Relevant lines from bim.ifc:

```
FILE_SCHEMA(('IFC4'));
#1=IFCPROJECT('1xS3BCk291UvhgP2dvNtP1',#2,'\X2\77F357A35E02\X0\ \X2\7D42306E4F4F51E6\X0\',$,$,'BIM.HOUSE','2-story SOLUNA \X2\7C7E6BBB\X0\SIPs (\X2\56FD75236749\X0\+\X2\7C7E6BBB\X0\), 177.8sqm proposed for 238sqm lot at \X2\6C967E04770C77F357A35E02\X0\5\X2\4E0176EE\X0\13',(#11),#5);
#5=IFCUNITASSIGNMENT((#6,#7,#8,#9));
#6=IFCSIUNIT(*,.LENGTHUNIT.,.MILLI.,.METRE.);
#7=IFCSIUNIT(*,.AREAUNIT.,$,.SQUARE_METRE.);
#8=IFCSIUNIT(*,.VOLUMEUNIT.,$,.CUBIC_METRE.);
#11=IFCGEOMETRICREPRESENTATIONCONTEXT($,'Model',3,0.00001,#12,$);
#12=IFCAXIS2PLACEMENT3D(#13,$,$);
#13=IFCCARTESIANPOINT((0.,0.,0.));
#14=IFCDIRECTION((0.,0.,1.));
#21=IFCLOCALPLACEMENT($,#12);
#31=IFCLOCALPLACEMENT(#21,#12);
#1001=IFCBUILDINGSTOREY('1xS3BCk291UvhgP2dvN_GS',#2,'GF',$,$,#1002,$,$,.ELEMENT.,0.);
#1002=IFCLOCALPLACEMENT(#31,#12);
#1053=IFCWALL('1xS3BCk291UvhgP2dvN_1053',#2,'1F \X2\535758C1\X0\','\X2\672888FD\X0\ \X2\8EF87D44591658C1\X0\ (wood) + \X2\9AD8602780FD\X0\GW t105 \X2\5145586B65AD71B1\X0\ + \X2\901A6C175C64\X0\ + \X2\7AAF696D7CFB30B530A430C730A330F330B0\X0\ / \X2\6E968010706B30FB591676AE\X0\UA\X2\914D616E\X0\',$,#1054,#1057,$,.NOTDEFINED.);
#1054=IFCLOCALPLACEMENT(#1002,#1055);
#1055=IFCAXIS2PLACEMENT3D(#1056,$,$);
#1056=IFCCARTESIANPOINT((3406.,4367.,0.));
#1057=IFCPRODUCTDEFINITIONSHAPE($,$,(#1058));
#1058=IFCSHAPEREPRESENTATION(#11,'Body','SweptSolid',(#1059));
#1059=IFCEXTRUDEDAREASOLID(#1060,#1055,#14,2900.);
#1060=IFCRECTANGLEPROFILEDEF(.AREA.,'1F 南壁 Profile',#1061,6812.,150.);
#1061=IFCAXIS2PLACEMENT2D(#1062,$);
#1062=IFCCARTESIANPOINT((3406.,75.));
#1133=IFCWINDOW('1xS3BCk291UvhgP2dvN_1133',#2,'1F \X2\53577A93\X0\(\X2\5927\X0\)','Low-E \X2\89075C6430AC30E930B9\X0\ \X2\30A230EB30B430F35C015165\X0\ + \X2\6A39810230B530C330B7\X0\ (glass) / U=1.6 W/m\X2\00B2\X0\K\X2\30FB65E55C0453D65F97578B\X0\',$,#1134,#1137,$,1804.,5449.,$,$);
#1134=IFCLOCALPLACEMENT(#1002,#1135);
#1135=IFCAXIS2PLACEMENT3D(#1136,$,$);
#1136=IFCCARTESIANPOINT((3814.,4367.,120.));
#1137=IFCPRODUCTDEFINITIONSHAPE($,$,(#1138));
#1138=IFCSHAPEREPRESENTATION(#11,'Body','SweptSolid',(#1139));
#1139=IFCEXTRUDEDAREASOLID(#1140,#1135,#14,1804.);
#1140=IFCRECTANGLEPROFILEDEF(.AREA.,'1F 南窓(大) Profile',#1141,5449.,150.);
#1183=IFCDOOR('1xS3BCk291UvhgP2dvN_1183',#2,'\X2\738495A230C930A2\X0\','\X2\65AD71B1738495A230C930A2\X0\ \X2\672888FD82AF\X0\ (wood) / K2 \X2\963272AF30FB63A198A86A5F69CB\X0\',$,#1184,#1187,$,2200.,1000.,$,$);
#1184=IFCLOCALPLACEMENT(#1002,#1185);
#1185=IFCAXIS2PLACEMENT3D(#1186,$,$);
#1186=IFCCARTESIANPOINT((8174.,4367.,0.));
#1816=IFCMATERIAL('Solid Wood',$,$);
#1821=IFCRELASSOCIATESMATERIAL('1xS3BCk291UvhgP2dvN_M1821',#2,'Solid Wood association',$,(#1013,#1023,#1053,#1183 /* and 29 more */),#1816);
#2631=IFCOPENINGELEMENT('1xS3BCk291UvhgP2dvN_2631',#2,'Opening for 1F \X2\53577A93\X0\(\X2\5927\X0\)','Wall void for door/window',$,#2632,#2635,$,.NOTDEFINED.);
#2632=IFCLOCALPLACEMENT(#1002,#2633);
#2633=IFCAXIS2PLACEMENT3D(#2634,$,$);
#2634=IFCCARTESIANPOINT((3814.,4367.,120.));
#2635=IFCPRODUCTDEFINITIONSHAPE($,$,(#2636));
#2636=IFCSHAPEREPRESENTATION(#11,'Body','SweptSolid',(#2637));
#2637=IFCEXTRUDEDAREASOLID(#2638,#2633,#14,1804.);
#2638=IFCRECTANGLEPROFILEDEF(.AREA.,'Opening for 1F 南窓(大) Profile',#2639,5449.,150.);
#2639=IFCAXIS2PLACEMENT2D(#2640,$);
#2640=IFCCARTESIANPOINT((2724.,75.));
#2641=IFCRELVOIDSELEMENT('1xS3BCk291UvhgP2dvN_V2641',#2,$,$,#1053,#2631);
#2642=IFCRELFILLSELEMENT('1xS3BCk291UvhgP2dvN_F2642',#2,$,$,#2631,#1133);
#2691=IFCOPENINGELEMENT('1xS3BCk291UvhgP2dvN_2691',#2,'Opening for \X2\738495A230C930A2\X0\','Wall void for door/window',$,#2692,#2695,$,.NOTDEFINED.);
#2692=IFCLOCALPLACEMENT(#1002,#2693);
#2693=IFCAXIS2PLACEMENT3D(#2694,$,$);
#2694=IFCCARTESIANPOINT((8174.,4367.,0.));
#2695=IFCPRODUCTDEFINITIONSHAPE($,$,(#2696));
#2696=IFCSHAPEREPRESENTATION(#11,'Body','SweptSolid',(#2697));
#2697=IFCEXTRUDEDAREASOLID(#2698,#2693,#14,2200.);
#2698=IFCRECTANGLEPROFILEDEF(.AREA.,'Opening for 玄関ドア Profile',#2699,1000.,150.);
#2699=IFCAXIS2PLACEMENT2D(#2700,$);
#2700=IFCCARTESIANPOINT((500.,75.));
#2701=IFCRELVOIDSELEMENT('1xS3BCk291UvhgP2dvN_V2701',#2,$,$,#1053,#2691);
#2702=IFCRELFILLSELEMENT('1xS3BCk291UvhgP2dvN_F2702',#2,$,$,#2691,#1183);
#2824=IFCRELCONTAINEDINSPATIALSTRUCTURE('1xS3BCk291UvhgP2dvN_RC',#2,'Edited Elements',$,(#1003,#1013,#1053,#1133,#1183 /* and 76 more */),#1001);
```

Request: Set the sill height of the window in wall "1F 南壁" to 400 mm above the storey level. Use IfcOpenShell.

```python
import numpy as np
import ifcopenshell
import ifcopenshell.api.geometry
import ifcopenshell.geom
import ifcopenshell.util.element
import ifcopenshell.util.placement
import ifcopenshell.util.shape
import ifcopenshell.util.unit

model = ifcopenshell.open("bim.ifc")
unit_scale = ifcopenshell.util.unit.calculate_unit_scale(model)

window = model.by_guid("1xS3BCk291UvhgP2dvN_1133")
opening = window.FillsVoids[0].RelatingOpeningElement
storey = ifcopenshell.util.element.get_container(window, ifc_class="IfcBuildingStorey")
level = ifcopenshell.util.placement.get_local_placement(storey.ObjectPlacement)[2, 3]

# The opening's origin need not be at the sill, so measure its lowest point.
shape = ifcopenshell.geom.create_shape(ifcopenshell.geom.settings(), opening)
bottom = ifcopenshell.util.shape.get_shape_bottom_elevation(shape, shape.geometry) / unit_scale
dz = level + 400.0 - bottom

shift = np.array([0.0, 0.0, dz])
# The window is not placed relative to its opening, so move both.
for product in (opening, window):
    matrix = ifcopenshell.util.placement.get_local_placement(product.ObjectPlacement)
    matrix[:3, 3] += shift
    ifcopenshell.api.geometry.edit_object_placement(model, product=product, matrix=matrix, is_si=False)

print(f"moved by {dz * unit_scale:+.3f} m")

model.write("bim_rev.ifc")
```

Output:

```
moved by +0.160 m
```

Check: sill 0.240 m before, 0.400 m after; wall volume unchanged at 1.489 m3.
